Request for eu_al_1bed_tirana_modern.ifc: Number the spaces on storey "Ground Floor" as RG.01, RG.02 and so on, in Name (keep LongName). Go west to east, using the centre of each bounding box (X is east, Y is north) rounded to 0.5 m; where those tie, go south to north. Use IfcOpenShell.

First a look at what the model holds.

```python
import ifcopenshell
import ifcopenshell.util.element
import ifcopenshell.util.placement

model = ifcopenshell.open("eu_al_1bed_tirana_modern.ifc")
print(model.schema)
storey = next(s for s in model.by_type("IfcBuildingStorey") if s.Name == "Ground Floor")
spaces = [e for e in ifcopenshell.util.element.get_decomposition(storey) if e.is_a("IfcSpace")]
for e in sorted(spaces, key=lambda e: e.id()):
    origin = ifcopenshell.util.placement.get_local_placement(e.ObjectPlacement)[:3, 3]
    print(e.id(), e.Name, e.LongName, origin.round(2) + 0.0, sep=" | ")
```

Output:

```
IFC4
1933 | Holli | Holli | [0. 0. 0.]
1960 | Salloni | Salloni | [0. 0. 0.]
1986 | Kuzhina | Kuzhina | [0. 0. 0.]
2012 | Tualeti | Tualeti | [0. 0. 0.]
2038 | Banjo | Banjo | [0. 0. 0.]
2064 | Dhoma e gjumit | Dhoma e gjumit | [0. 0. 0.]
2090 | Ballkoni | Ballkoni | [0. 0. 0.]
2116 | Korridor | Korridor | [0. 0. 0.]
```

```python
import ifcopenshell
import ifcopenshell.geom
import ifcopenshell.util.element
import ifcopenshell.util.shape

model = ifcopenshell.open("eu_al_1bed_tirana_modern.ifc")
settings = ifcopenshell.geom.settings()
settings.set("use-world-coords", True)


def centre(element):
    shape = ifcopenshell.geom.create_shape(settings, element)
    return ifcopenshell.util.shape.get_bbox_centroid(shape.geometry)


storey = next(s for s in model.by_type("IfcBuildingStorey") if s.Name == "Ground Floor")
spaces = [e for e in ifcopenshell.util.element.get_decomposition(storey) if e.is_a("IfcSpace")]

# Insertion points can sit at a corner or the storey origin, so sort by the geometry (in metres).
centres = {e: centre(e) for e in spaces}
spaces.sort(key=lambda e: (round(centres[e][0] / 0.5), centres[e][1]))

for i, e in enumerate(spaces, start=1):
    number = f"RG.{i:02d}"
    e.Name = number
    print(e.id(), number)

model.write("eu_al_1bed_tirana_modern_updated.ifc")
```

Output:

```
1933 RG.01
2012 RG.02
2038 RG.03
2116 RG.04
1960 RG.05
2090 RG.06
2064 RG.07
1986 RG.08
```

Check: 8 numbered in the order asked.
